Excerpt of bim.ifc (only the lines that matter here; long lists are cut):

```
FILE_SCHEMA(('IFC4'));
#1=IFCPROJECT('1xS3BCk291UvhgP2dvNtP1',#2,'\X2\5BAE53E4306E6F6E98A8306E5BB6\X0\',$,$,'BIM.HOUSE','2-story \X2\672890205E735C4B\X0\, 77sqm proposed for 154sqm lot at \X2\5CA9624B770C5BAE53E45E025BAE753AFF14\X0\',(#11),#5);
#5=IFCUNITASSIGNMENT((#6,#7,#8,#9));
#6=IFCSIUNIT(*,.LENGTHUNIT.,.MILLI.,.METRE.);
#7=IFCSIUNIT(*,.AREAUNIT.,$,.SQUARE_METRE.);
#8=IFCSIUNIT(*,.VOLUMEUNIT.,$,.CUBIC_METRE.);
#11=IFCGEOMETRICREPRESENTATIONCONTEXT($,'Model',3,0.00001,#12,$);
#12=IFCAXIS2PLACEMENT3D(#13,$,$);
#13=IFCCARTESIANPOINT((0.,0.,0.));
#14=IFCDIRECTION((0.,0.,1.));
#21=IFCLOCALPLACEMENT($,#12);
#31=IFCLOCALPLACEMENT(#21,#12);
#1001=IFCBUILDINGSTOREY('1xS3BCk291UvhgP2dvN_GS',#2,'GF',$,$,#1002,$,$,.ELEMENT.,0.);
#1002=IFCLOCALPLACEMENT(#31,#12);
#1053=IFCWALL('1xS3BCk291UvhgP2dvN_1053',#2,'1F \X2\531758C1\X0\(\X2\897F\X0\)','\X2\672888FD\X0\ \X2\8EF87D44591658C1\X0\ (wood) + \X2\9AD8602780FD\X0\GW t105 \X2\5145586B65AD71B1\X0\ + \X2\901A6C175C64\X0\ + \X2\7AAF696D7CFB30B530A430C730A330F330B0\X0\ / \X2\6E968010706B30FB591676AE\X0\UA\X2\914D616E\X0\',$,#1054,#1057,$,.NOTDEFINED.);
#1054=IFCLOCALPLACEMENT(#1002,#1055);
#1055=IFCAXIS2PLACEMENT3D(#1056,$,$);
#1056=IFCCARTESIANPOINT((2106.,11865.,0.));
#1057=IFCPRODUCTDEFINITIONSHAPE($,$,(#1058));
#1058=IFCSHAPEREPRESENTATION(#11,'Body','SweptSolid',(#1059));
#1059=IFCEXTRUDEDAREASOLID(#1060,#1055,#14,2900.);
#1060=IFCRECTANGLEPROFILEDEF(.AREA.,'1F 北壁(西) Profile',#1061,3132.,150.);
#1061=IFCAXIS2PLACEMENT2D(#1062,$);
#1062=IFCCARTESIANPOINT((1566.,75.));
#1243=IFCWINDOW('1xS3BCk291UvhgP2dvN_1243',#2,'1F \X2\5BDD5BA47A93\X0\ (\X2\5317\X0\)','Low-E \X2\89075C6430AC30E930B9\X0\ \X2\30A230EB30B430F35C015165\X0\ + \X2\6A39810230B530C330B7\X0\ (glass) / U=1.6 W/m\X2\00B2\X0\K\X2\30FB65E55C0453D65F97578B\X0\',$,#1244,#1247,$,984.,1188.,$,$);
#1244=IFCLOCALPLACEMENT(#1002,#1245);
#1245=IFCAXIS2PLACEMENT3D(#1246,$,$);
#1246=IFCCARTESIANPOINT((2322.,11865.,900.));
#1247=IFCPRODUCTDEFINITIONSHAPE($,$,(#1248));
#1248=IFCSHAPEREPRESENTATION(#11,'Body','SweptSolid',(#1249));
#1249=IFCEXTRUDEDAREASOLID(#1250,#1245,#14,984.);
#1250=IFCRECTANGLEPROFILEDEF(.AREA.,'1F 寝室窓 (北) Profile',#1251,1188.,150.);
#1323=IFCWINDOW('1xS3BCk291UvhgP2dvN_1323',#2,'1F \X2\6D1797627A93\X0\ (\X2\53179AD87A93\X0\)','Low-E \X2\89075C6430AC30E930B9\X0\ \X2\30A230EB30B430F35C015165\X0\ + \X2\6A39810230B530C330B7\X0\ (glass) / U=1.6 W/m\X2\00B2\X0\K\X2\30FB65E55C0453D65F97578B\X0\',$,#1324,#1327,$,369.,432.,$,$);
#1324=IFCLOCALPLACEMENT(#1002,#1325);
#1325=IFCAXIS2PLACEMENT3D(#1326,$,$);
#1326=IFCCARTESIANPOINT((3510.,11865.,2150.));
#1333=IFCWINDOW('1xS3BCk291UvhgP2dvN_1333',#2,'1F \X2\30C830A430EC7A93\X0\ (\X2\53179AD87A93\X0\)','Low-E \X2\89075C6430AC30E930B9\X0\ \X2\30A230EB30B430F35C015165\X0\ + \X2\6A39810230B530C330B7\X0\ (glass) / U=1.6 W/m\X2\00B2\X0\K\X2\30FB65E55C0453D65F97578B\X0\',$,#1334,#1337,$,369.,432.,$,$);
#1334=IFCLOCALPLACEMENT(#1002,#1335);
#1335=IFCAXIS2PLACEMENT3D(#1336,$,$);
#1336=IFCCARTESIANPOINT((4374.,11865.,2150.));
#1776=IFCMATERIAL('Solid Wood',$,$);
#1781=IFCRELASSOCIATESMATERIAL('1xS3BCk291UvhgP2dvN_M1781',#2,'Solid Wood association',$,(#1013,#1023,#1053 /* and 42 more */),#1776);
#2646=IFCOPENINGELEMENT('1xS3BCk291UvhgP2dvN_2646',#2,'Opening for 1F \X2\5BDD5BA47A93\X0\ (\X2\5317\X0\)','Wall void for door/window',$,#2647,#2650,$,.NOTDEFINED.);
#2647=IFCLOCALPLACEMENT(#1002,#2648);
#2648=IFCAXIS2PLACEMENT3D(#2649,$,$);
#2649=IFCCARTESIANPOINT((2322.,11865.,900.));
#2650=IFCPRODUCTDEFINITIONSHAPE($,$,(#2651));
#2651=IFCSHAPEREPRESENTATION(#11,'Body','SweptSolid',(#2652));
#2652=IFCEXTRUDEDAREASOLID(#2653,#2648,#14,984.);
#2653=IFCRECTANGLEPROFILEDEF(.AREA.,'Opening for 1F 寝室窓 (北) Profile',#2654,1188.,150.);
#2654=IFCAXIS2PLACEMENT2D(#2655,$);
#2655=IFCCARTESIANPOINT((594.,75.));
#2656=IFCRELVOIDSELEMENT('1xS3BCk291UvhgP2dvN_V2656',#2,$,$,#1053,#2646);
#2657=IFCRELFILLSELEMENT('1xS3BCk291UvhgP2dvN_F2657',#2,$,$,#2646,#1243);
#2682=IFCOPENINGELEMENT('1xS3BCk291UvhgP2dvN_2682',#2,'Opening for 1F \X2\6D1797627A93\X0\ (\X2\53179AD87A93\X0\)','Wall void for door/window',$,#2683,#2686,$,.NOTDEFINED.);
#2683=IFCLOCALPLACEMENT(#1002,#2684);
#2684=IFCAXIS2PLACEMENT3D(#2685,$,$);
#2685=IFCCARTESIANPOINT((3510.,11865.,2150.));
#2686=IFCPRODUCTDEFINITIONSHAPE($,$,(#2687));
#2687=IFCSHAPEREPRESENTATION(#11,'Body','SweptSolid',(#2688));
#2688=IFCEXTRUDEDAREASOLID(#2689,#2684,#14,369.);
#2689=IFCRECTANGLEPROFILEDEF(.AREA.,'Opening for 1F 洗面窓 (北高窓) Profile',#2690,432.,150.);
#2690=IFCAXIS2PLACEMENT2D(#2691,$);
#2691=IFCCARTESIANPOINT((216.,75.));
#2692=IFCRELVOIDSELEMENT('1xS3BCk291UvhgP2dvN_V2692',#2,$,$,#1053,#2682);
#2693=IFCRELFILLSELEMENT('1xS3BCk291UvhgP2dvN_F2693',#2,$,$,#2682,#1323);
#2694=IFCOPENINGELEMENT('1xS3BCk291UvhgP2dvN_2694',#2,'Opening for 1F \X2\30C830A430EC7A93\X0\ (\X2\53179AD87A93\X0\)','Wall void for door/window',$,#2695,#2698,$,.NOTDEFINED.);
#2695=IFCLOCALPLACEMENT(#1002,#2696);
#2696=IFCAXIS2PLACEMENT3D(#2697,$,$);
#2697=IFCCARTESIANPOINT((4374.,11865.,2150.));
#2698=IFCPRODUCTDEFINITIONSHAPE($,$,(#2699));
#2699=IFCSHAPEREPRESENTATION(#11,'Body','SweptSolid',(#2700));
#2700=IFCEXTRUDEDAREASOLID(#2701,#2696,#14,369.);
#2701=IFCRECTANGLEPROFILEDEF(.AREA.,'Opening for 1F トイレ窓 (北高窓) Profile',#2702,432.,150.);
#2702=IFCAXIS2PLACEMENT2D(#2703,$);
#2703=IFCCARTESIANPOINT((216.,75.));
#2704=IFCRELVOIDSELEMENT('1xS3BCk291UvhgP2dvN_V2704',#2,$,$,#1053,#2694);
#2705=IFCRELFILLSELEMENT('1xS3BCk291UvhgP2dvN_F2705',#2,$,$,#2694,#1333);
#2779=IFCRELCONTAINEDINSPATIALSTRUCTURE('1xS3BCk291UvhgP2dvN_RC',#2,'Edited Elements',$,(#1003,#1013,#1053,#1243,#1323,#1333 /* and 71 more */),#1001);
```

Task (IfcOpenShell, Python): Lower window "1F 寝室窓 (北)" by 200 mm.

```python
import numpy as np
import ifcopenshell
import ifcopenshell.api.geometry
import ifcopenshell.util.placement
import ifcopenshell.util.unit

model = ifcopenshell.open("bim.ifc")
unit_scale = ifcopenshell.util.unit.calculate_unit_scale(model)

window = model.by_id(1243)
opening = window.FillsVoids[0].RelatingOpeningElement
dz = -200.0

shift = np.array([0.0, 0.0, dz])
# The window is not placed relative to its opening, so move both.
for product in (opening, window):
    matrix = ifcopenshell.util.placement.get_local_placement(product.ObjectPlacement)
    matrix[:3, 3] += shift
    ifcopenshell.api.geometry.edit_object_placement(model, product=product, matrix=matrix, is_si=False)

print(f"moved by {dz * unit_scale:+.3f} m")

model.write("bim_edited.ifc")
```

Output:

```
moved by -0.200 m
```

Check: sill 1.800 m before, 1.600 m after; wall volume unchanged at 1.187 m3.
